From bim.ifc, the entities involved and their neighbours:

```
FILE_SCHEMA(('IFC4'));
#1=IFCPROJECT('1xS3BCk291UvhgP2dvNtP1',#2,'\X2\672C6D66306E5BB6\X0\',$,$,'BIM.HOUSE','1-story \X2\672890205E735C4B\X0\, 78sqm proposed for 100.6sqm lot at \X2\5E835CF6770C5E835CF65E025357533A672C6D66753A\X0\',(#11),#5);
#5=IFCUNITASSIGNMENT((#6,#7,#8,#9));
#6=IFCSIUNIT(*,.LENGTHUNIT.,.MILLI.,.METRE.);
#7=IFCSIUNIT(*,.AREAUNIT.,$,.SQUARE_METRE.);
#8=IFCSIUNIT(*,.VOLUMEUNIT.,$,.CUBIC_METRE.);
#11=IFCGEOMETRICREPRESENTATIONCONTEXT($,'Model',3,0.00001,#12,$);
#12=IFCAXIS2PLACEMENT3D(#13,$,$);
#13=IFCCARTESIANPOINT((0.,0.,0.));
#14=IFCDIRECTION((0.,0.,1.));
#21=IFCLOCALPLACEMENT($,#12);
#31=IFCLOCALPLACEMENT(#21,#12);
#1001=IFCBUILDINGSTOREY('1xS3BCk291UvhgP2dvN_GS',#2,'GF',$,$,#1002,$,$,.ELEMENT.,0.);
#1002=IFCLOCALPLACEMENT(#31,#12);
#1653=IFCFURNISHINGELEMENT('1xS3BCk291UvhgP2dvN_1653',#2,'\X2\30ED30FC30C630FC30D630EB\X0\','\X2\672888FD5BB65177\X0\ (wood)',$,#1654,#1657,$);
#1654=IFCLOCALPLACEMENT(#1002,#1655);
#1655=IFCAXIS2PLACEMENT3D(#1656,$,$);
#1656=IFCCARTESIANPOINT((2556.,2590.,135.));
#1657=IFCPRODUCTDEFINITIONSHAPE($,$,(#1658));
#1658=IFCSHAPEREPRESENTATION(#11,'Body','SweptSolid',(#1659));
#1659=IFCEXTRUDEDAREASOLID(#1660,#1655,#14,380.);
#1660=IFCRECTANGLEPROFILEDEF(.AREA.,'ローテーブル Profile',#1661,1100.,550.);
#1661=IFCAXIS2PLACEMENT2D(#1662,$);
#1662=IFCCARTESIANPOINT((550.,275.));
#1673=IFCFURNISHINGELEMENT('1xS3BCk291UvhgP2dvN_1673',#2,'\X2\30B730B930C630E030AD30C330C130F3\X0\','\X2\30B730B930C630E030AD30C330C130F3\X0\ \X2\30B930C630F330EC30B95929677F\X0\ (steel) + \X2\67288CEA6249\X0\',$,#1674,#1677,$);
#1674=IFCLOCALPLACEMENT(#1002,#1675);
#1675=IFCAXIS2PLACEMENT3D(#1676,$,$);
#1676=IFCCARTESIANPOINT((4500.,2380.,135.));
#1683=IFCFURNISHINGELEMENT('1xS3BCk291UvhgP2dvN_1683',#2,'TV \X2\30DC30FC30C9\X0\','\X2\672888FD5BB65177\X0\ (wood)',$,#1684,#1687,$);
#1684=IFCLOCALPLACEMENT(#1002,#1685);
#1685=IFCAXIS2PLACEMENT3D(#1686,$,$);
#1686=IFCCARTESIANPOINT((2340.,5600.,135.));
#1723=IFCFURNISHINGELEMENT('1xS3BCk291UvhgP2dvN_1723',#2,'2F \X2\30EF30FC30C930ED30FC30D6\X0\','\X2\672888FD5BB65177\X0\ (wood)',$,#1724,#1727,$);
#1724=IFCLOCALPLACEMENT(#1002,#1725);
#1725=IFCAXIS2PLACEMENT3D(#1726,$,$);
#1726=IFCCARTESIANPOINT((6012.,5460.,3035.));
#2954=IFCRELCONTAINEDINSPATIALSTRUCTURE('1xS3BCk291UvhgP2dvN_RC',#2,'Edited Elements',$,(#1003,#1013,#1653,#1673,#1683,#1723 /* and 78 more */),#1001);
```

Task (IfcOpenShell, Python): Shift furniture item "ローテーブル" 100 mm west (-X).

```python
import ifcopenshell
import ifcopenshell.api.geometry
import ifcopenshell.util.placement

model = ifcopenshell.open("bim.ifc")

item = model.by_guid("1xS3BCk291UvhgP2dvN_1653")
matrix = ifcopenshell.util.placement.get_local_placement(item.ObjectPlacement)
matrix[0, 3] -= 100.0
ifcopenshell.api.geometry.edit_object_placement(model, product=item, matrix=matrix, is_si=False)

print(ifcopenshell.util.placement.get_local_placement(item.ObjectPlacement).round(3) + 0.0)

model.write("bim-out.ifc")
```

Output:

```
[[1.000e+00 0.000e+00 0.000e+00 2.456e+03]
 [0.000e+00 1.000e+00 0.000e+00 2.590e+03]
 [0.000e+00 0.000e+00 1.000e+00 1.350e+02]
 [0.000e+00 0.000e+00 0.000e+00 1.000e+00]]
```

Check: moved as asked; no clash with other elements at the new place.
